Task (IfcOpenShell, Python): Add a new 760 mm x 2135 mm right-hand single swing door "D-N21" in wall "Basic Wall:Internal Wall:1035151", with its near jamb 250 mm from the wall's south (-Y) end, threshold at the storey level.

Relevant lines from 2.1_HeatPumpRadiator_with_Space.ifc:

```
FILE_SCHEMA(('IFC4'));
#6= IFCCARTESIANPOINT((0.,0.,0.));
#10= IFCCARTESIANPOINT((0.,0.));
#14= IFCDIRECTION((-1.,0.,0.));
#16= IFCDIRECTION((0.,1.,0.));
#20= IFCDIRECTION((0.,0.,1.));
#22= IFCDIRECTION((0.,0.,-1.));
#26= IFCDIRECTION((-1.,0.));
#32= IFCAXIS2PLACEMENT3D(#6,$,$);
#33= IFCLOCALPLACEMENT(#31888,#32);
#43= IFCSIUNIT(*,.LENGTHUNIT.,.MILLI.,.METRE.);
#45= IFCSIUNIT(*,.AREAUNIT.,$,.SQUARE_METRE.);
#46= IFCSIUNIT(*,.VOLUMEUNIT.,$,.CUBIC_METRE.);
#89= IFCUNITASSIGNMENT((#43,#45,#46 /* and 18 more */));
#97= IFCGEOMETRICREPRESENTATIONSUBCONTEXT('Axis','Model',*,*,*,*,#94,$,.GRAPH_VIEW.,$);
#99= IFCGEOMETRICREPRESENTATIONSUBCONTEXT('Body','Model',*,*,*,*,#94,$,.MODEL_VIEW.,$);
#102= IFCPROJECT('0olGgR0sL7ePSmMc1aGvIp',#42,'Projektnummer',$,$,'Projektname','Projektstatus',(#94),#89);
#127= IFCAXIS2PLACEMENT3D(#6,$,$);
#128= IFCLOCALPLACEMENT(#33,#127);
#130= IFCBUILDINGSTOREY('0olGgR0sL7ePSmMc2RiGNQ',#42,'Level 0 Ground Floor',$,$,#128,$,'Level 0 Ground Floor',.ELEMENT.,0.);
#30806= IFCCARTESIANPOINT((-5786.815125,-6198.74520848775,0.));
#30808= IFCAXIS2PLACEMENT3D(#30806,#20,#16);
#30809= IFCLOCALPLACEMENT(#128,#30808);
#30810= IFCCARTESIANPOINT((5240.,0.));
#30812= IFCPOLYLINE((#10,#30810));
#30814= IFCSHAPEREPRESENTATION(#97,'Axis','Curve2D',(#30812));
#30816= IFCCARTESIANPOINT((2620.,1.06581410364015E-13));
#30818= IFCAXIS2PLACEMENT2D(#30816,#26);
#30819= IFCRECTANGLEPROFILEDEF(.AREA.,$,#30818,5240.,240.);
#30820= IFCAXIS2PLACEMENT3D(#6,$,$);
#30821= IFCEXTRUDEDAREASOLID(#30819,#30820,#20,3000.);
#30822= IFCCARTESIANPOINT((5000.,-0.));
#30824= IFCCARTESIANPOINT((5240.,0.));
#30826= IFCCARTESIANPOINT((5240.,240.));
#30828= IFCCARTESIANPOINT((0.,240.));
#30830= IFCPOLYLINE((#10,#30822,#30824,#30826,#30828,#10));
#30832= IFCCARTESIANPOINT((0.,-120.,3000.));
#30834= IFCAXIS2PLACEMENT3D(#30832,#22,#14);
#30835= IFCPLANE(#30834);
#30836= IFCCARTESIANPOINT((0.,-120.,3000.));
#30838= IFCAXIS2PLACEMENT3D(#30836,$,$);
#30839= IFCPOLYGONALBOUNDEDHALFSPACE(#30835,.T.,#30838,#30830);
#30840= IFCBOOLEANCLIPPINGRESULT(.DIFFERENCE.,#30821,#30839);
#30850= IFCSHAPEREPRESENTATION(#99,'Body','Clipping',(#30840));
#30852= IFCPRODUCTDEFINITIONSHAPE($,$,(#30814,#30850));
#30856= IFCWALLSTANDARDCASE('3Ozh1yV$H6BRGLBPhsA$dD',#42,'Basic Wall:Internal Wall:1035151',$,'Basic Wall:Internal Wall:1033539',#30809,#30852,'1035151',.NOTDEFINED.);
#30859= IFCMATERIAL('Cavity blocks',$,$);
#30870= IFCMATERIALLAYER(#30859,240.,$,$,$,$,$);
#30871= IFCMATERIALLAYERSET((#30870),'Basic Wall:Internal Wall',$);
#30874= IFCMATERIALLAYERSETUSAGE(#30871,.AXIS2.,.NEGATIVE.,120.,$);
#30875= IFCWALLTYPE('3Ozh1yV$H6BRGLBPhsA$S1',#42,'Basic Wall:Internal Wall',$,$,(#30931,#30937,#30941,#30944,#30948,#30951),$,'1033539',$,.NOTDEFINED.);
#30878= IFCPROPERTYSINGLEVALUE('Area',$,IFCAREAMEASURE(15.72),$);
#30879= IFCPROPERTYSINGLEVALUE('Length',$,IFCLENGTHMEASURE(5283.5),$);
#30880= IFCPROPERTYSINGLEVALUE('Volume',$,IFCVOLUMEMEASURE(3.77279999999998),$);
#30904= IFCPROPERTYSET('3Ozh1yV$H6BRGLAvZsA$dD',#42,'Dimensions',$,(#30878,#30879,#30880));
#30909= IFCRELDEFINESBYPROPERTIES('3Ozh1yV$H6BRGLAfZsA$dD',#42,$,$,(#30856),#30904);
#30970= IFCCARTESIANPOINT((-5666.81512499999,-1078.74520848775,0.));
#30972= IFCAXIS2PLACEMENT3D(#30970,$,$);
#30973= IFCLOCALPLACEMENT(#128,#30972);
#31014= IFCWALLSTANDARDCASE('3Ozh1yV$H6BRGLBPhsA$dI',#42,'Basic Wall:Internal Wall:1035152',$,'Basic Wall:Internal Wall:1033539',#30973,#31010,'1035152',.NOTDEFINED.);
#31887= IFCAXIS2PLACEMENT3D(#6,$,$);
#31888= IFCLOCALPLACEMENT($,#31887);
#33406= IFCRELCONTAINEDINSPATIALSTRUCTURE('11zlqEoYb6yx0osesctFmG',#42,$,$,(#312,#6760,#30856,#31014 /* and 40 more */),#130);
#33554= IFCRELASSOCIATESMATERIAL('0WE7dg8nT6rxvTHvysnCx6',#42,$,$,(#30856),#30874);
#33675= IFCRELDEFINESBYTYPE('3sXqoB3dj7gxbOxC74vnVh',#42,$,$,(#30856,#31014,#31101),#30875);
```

```python
import numpy as np
import ifcopenshell
import ifcopenshell.api.feature
import ifcopenshell.api.geometry
import ifcopenshell.api.pset
import ifcopenshell.api.root
import ifcopenshell.api.spatial
import ifcopenshell.geom
import ifcopenshell.util.element
import ifcopenshell.util.placement
import ifcopenshell.util.representation
import ifcopenshell.util.shape
import ifcopenshell.util.unit

model = ifcopenshell.open("2.1_HeatPumpRadiator_with_Space.ifc")
unit_scale = ifcopenshell.util.unit.calculate_unit_scale(model)
area_scale = ifcopenshell.util.unit.calculate_unit_scale(model, "AREAUNIT")
volume_scale = ifcopenshell.util.unit.calculate_unit_scale(model, "VOLUMEUNIT")
settings = ifcopenshell.geom.settings()


def volume(element):
    """Net volume in cubic metres, openings subtracted."""
    shape = ifcopenshell.geom.create_shape(settings, element)
    return ifcopenshell.util.shape.get_volume(shape.geometry)


wall = model.by_guid("3Ozh1yV$H6BRGLBPhsA$dD")
storey = ifcopenshell.util.element.get_container(wall, ifc_class="IfcBuildingStorey")
context = ifcopenshell.util.representation.get_context(model, "Model", "Body", "MODEL_VIEW")
before = volume(wall)

width, height, from_end, sill = 0.76, 2.135, 0.25, 0.0  # metres

# The wall runs along its own X axis, and the end named is its -X end.
wall_shape = ifcopenshell.geom.create_shape(settings, wall)
x, y, z = ifcopenshell.util.shape.get_vertices(wall_shape.geometry).T
start = x.min() + from_end
face, thickness = float(y.min()), float(y.max() - y.min())
wall_matrix = ifcopenshell.util.placement.get_local_placement(wall.ObjectPlacement)
level = ifcopenshell.util.placement.get_local_placement(storey.ObjectPlacement)[2, 3]


def in_wall(x, y):
    """Placement at x, y metres in the wall's axes, at sill height."""
    matrix = wall_matrix.copy()
    matrix[:, 3] = wall_matrix @ np.array([x / unit_scale, y / unit_scale, 0.0, 1.0])
    matrix[2, 3] = level + sill / unit_scale
    return matrix


# Opening: a box that overshoots both wall faces by 50 mm.
opening = ifcopenshell.api.root.create_entity(model, ifc_class="IfcOpeningElement", predefined_type="OPENING")
box = ifcopenshell.api.geometry.add_wall_representation(
    model, context=context, length=width, height=height, thickness=thickness + 0.1
)
ifcopenshell.api.geometry.assign_representation(model, product=opening, representation=box)
ifcopenshell.api.geometry.edit_object_placement(model, product=opening, matrix=in_wall(start, face - 0.05), is_si=False)
ifcopenshell.api.feature.add_feature(model, feature=opening, element=wall)

door = ifcopenshell.api.root.create_entity(model, ifc_class="IfcDoor", name="D-N21", predefined_type="DOOR")
door.OverallWidth, door.OverallHeight = width / unit_scale, height / unit_scale
door.OperationType = "SINGLE_SWING_RIGHT"
body = ifcopenshell.api.geometry.add_door_representation(
    model,
    context=context,
    overall_width=door.OverallWidth,
    overall_height=door.OverallHeight,
    operation_type="SINGLE_SWING_RIGHT",
    lining_properties={"LiningDepth": thickness / unit_scale, "ThresholdDepth": thickness / unit_scale},
)
ifcopenshell.api.geometry.assign_representation(model, product=door, representation=body)
ifcopenshell.api.spatial.assign_container(model, products=[door], relating_structure=storey)
ifcopenshell.api.feature.add_filling(model, opening=opening, element=door)

# The lining spans the wall, so the door starts at the wall face.
ifcopenshell.api.geometry.edit_object_placement(model, product=door, matrix=in_wall(start, face), is_si=False)

after = volume(wall)

# Update the wall's stored quantities.
pset = model.by_id(ifcopenshell.util.element.get_pset(wall, "Dimensions", should_inherit=False)["id"])
ifcopenshell.api.pset.edit_pset(model, pset=pset, properties={
    "Area": model.create_entity("IfcAreaMeasure", after / thickness / area_scale),
    "Volume": model.create_entity("IfcVolumeMeasure", after / volume_scale),
})

print(f"wall volume {before:.3f} -> {after:.3f} m3")

model.write("2.1_HeatPumpRadiator_with_Space_rev.ifc")
```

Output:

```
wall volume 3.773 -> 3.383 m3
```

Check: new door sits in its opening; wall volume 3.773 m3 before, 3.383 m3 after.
